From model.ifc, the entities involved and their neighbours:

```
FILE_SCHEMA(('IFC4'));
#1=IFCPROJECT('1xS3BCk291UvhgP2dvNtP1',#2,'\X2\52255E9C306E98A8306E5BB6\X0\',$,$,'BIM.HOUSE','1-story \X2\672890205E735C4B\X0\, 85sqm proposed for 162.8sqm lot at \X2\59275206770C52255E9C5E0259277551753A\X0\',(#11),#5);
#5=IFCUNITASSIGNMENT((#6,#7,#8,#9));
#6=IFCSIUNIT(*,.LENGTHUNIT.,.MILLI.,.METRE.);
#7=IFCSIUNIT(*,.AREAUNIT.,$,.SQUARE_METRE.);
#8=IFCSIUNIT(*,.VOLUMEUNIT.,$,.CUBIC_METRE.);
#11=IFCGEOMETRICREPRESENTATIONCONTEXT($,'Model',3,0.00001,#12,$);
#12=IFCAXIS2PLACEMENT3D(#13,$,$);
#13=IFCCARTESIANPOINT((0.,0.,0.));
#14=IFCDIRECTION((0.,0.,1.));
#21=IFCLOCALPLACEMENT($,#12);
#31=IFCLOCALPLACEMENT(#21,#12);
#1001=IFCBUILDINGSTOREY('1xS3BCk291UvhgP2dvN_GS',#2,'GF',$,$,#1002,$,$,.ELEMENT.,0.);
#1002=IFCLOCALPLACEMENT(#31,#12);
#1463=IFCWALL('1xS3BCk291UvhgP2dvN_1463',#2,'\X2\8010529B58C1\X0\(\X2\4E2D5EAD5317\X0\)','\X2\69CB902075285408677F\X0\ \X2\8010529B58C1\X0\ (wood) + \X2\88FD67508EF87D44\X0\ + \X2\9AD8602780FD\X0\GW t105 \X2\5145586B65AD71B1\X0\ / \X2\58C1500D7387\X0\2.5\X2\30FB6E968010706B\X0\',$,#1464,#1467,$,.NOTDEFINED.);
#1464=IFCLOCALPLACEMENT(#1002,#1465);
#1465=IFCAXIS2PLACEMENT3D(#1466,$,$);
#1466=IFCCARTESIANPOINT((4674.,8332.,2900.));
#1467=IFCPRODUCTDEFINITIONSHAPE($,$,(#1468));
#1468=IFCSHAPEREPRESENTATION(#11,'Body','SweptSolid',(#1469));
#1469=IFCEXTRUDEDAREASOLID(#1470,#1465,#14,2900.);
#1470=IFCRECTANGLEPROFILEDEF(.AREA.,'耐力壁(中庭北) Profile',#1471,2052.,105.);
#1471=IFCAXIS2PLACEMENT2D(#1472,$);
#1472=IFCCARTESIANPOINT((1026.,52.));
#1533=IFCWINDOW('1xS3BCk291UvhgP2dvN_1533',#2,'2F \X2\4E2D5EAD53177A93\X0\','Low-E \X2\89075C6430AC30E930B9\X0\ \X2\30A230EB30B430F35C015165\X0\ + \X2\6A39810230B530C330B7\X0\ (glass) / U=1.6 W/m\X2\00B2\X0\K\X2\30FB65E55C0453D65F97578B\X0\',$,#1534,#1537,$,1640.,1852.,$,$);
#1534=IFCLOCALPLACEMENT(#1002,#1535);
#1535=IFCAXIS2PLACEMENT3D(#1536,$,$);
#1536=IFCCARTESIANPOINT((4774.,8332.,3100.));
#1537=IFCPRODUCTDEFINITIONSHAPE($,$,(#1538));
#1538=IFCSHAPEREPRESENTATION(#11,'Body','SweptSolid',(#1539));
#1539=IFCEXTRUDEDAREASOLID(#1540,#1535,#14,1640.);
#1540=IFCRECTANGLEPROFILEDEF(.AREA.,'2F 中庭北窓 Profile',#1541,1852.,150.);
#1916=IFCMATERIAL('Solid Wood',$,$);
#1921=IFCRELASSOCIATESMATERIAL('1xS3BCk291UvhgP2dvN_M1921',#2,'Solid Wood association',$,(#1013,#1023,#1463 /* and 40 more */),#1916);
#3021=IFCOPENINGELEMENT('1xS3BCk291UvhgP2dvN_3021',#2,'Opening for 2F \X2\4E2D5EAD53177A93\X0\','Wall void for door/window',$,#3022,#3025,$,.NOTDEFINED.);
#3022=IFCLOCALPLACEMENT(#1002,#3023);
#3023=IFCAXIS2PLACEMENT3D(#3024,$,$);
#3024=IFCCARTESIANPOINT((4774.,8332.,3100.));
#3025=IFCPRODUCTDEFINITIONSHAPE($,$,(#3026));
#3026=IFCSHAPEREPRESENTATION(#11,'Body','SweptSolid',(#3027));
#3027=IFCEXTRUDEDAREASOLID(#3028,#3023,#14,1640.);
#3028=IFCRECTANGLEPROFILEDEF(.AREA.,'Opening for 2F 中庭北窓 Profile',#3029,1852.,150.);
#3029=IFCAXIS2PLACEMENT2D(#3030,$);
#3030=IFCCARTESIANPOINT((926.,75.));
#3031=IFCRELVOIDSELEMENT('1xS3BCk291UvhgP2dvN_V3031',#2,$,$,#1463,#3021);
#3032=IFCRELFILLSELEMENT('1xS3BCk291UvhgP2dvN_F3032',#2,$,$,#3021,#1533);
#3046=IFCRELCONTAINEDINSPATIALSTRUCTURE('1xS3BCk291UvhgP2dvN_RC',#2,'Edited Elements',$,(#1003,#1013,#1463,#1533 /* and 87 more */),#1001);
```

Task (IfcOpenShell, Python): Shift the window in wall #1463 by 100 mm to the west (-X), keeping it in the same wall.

```python
import ifcopenshell
import ifcopenshell.api.geometry
import ifcopenshell.util.placement

model = ifcopenshell.open("model.ifc")

window = model.by_guid("1xS3BCk291UvhgP2dvN_1533")
opening = window.FillsVoids[0].RelatingOpeningElement
wall = opening.VoidsElements[0].RelatingBuildingElement

wall_matrix = ifcopenshell.util.placement.get_local_placement(wall.ObjectPlacement)
shift = wall_matrix[:3, 0] * -100.0
before = ifcopenshell.util.placement.get_local_placement(window.ObjectPlacement)[:3, 3].copy()

# The window is not placed relative to its opening, so move both.
for product in (opening, window):
    matrix = ifcopenshell.util.placement.get_local_placement(product.ObjectPlacement)
    matrix[:3, 3] += shift
    ifcopenshell.api.geometry.edit_object_placement(model, product=product, matrix=matrix, is_si=False)

after = ifcopenshell.util.placement.get_local_placement(window.ObjectPlacement)[:3, 3]
print("window moved by", (after - before).round(3) + 0.0)

model.write("model-out.ifc")
```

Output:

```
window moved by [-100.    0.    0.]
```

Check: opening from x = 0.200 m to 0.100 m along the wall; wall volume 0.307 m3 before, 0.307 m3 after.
